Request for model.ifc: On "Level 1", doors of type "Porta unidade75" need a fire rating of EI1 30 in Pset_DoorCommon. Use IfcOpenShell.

First a look at what the model holds.

```python
import ifcopenshell
import ifcopenshell.util.element

model = ifcopenshell.open("model.ifc")
print(model.schema)
storey = next(s for s in model.by_type("IfcBuildingStorey") if s.Name == "Level 1")
doors = [e for e in ifcopenshell.util.element.get_decomposition(storey) if e.is_a("IfcDoor")]
seen = {}
for e in doors:
    element_type = ifcopenshell.util.element.get_type(e)
    key = (element_type.Name if element_type != e and element_type else None, ifcopenshell.util.element.get_pset(e, "Pset_DoorCommon", "FireRating"))
    seen[key] = seen.get(key, 0) + 1
for (name, value), count in sorted(seen.items(), key=str):
    print(count, "x", name, "|", value)
```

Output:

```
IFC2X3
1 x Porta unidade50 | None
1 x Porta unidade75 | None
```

```python
import ifcopenshell
import ifcopenshell.api.pset
import ifcopenshell.util.element

model = ifcopenshell.open("model.ifc")

storey = next(s for s in model.by_type("IfcBuildingStorey") if s.Name == "Level 1")
doors = [e for e in ifcopenshell.util.element.get_decomposition(storey) if e.is_a("IfcDoor")]

count = 0
for e in doors:
    element_type = ifcopenshell.util.element.get_type(e)
    if element_type in (None, e) or element_type.Name != "Porta unidade75":
        continue
    # add_pset returns the element's existing set when there is one.
    pset = ifcopenshell.api.pset.add_pset(model, product=e, name="Pset_DoorCommon")
    ifcopenshell.api.pset.edit_pset(model, pset=pset, properties={"FireRating": "EI1 30"})
    count += 1

print(count, "doors updated")

model.write("model-out.ifc")
```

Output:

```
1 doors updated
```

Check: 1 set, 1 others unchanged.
